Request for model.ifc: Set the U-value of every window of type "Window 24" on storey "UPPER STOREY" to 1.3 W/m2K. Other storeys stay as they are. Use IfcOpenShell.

First a look at what the model holds.

```python
import ifcopenshell
import ifcopenshell.util.element

model = ifcopenshell.open("model.ifc")
print(model.schema)
storey = next(s for s in model.by_type("IfcBuildingStorey") if s.Name == "UPPER STOREY")
windows = [e for e in ifcopenshell.util.element.get_decomposition(storey) if e.is_a("IfcWindow")]
seen = {}
for e in windows:
    element_type = ifcopenshell.util.element.get_type(e)
    key = (element_type.Name if element_type != e and element_type else None, ifcopenshell.util.element.get_pset(e, "Pset_WindowCommon", "ThermalTransmittance"))
    seen[key] = seen.get(key, 0) + 1
for (name, value), count in sorted(seen.items(), key=str):
    print(count, "x", name, "|", value)
```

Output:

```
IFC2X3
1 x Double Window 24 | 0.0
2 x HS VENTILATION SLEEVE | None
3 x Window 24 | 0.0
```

```python
import ifcopenshell
import ifcopenshell.api.pset
import ifcopenshell.util.element

model = ifcopenshell.open("model.ifc")

storey = next(s for s in model.by_type("IfcBuildingStorey") if s.Name == "UPPER STOREY")
windows = [e for e in ifcopenshell.util.element.get_decomposition(storey) if e.is_a("IfcWindow")]

count = 0
for e in windows:
    element_type = ifcopenshell.util.element.get_type(e)
    if element_type in (None, e) or element_type.Name != "Window 24":
        continue
    # add_pset returns the element's existing set when there is one.
    pset = ifcopenshell.api.pset.add_pset(model, product=e, name="Pset_WindowCommon")
    ifcopenshell.api.pset.edit_pset(model, pset=pset, properties={"ThermalTransmittance": 1.3})
    count += 1

print(count, "windows updated")

model.write("model_edited.ifc")
```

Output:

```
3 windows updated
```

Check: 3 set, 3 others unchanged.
